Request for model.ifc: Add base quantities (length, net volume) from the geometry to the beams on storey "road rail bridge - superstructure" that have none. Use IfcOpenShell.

First a look at what the model holds.

```python
import ifcopenshell
import ifcopenshell.util.element
import ifcopenshell.util.unit

model = ifcopenshell.open("model.ifc")
print(model.schema)
for unit_type in ("LENGTHUNIT", "AREAUNIT", "VOLUMEUNIT"):
    print(unit_type, ifcopenshell.util.unit.calculate_unit_scale(model, unit_type))
storey = next(s for s in model.by_type("IfcBuildingStorey") if s.Name == "road rail bridge - superstructure")
beams = [e for e in ifcopenshell.util.element.get_decomposition(storey) if e.is_a("IfcBeam")]
for e in sorted(beams, key=lambda e: e.id()):
    print(e.id(), e.is_a(), e.Name, list(ifcopenshell.util.element.get_psets(e, qtos_only=True)), sep=" | ")
```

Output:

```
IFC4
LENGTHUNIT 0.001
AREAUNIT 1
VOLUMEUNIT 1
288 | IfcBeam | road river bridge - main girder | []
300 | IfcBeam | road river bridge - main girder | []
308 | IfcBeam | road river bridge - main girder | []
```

```python
import ifcopenshell
import ifcopenshell.api.pset
import ifcopenshell.geom
import ifcopenshell.util.element
import ifcopenshell.util.shape
import ifcopenshell.util.unit

model = ifcopenshell.open("model.ifc")
unit_scale = ifcopenshell.util.unit.calculate_unit_scale(model)
volume_scale = ifcopenshell.util.unit.calculate_unit_scale(model, "VOLUMEUNIT")
settings = ifcopenshell.geom.settings()

storey = next(s for s in model.by_type("IfcBuildingStorey") if s.Name == "road rail bridge - superstructure")
beams = [e for e in ifcopenshell.util.element.get_decomposition(storey) if e.is_a("IfcBeam")]

for e in sorted(beams, key=lambda e: e.id()):
    if ifcopenshell.util.element.get_psets(e, qtos_only=True, should_inherit=False):
        continue
    # Geometry comes back in metres, in the element's own axes.
    shape = ifcopenshell.geom.create_shape(settings, e)
    values = {
        "Length": ifcopenshell.util.shape.get_max_xyz(shape.geometry) / unit_scale,
        "NetVolume": ifcopenshell.util.shape.get_volume(shape.geometry) / volume_scale,
    }
    qto = ifcopenshell.api.pset.add_qto(model, product=e, name="Qto_BeamBaseQuantities")
    ifcopenshell.api.pset.edit_qto(model, qto=qto, properties=values)
    print(e.id(), {k: round(v, 3) for k, v in values.items()})

model.write("model_v2.ifc")
```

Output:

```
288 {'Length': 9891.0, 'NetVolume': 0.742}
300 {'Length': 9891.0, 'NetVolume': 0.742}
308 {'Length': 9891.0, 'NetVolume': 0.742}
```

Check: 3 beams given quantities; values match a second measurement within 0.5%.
